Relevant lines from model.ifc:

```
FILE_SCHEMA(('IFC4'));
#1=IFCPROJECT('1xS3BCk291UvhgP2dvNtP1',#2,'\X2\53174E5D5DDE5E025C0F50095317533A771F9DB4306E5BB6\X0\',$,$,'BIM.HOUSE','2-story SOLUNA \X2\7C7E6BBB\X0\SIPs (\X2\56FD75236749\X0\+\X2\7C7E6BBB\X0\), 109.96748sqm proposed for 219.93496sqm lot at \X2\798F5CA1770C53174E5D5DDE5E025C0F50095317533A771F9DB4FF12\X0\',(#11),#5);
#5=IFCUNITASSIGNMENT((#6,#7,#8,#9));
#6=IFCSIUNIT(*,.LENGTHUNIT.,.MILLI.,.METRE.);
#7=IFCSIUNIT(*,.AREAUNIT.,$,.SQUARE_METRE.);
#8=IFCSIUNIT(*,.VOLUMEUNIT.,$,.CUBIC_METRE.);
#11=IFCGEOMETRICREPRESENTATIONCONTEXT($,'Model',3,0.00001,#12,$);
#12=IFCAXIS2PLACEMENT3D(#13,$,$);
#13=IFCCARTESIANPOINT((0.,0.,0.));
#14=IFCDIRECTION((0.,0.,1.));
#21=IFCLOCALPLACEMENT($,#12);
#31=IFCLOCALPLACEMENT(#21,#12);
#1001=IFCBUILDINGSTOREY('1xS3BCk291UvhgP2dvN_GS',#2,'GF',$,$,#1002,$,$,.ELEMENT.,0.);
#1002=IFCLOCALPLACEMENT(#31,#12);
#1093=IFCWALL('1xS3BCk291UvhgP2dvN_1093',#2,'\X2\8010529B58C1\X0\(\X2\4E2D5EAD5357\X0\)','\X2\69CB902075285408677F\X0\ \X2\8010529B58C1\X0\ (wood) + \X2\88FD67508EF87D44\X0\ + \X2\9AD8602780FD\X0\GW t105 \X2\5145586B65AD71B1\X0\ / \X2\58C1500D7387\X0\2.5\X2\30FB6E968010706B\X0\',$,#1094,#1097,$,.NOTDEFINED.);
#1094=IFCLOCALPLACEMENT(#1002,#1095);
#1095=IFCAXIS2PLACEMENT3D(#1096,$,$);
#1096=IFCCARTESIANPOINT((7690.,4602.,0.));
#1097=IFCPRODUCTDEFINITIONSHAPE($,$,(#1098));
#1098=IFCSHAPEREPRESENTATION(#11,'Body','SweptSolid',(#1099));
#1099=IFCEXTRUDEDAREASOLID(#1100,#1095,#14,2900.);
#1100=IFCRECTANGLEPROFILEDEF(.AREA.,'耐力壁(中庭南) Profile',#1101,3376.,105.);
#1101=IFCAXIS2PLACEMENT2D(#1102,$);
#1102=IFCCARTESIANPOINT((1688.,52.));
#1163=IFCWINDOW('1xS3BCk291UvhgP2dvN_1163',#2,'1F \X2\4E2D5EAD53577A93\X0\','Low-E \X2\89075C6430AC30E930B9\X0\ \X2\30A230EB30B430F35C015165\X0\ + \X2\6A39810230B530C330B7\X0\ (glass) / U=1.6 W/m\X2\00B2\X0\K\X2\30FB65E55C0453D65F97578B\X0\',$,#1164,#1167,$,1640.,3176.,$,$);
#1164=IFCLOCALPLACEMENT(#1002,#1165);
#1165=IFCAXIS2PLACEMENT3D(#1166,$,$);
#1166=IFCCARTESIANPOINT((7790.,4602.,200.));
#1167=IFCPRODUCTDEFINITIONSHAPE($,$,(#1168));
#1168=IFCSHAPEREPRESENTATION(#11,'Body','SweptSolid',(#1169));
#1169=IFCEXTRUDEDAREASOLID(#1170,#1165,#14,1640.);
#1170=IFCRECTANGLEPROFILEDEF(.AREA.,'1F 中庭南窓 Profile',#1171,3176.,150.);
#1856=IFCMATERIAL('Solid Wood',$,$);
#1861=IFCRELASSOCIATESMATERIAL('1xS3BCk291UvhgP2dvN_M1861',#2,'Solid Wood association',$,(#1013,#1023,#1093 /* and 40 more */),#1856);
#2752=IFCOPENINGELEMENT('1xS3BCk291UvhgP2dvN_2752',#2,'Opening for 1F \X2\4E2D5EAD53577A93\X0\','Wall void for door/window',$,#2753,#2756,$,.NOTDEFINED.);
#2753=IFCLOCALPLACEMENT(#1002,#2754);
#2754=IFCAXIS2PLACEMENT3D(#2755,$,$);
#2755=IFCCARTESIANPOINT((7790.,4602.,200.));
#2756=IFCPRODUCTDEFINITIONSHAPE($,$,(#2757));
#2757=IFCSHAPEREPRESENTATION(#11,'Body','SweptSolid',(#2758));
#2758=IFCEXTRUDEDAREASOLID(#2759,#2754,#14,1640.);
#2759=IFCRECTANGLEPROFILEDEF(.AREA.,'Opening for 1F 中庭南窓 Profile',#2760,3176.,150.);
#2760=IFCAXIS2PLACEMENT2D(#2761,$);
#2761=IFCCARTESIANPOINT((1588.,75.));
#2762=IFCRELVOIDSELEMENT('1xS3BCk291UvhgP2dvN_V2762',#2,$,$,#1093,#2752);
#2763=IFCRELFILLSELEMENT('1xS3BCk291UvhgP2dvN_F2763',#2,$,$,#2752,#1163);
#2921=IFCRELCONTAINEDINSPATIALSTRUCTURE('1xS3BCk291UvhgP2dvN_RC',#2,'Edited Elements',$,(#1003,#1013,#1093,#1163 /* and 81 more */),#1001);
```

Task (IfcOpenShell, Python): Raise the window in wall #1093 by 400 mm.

```python
import numpy as np
import ifcopenshell
import ifcopenshell.api.geometry
import ifcopenshell.util.placement
import ifcopenshell.util.unit

model = ifcopenshell.open("model.ifc")
unit_scale = ifcopenshell.util.unit.calculate_unit_scale(model)

window = model.by_id(1163)
opening = window.FillsVoids[0].RelatingOpeningElement
dz = 400.0

shift = np.array([0.0, 0.0, dz])
# The window is not placed relative to its opening, so move both.
for product in (opening, window):
    matrix = ifcopenshell.util.placement.get_local_placement(product.ObjectPlacement)
    matrix[:3, 3] += shift
    ifcopenshell.api.geometry.edit_object_placement(model, product=product, matrix=matrix, is_si=False)

print(f"moved by {dz * unit_scale:+.3f} m")

model.write("model_rev.ifc")
```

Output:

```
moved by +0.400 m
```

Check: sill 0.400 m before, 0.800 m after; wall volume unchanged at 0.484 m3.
